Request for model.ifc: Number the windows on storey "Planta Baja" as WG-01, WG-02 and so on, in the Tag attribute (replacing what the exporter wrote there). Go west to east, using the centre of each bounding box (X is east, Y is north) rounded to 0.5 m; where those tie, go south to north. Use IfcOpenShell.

First a look at what the model holds.

```python
import ifcopenshell
import ifcopenshell.util.element
import ifcopenshell.util.placement

model = ifcopenshell.open("model.ifc")
print(model.schema)
storey = next(s for s in model.by_type("IfcBuildingStorey") if s.Name == "Planta Baja")
windows = [e for e in ifcopenshell.util.element.get_decomposition(storey) if e.is_a("IfcWindow")]
for e in sorted(windows, key=lambda e: e.id()):
    origin = ifcopenshell.util.placement.get_local_placement(e.ObjectPlacement)[:3, 3]
    print(e.id(), e.Tag, e.Name, origin.round(2) + 0.0, sep=" | ")
```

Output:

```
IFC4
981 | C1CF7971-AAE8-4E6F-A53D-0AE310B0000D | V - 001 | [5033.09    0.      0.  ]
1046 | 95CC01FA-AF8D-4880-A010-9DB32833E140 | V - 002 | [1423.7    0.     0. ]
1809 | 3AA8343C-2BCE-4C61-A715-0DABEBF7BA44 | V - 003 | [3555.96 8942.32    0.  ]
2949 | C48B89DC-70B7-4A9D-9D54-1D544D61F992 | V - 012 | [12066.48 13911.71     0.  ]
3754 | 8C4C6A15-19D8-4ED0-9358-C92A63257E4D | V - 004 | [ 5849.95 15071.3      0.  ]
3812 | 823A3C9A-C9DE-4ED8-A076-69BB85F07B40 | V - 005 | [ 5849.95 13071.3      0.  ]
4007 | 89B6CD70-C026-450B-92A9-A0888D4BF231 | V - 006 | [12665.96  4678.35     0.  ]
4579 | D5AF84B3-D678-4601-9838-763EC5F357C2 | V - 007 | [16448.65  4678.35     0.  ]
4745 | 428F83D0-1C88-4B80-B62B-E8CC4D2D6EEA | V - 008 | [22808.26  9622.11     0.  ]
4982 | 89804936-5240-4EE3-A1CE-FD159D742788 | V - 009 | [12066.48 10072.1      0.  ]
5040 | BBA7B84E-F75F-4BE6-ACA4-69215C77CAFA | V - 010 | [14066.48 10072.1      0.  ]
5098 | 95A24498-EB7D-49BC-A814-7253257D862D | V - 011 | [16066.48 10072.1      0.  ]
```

```python
import ifcopenshell
import ifcopenshell.geom
import ifcopenshell.util.element
import ifcopenshell.util.shape

model = ifcopenshell.open("model.ifc")
settings = ifcopenshell.geom.settings()
settings.set("use-world-coords", True)


def centre(element):
    shape = ifcopenshell.geom.create_shape(settings, element)
    return ifcopenshell.util.shape.get_bbox_centroid(shape.geometry)


storey = next(s for s in model.by_type("IfcBuildingStorey") if s.Name == "Planta Baja")
windows = [e for e in ifcopenshell.util.element.get_decomposition(storey) if e.is_a("IfcWindow")]

# Insertion points can sit at a corner or the storey origin, so sort by the geometry (in metres).
centres = {e: centre(e) for e in windows}
windows.sort(key=lambda e: (round(centres[e][0] / 0.5), centres[e][1]))

for i, e in enumerate(windows, start=1):
    number = f"WG-{i:02d}"
    e.Tag = number
    print(e.id(), number)

model.write("model_v2.ifc")
```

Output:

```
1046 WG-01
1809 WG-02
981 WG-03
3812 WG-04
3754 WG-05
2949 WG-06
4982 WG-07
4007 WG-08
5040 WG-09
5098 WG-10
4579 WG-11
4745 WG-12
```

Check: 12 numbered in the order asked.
